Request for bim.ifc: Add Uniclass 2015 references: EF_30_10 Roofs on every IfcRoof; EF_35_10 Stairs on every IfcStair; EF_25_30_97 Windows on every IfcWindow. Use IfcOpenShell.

First a look at what the model holds.

```python
import ifcopenshell

model = ifcopenshell.open("bim.ifc")
print(model.schema)
print("classifications:", [c.Name for c in model.by_type("IfcClassification")])
for ifc_class in ("IfcDoor", "IfcRoof", "IfcStair", "IfcWall", "IfcWindow"):
    print(ifc_class, len(model.by_type(ifc_class)))
```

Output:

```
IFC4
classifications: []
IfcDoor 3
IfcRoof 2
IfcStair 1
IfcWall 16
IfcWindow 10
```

```python
import ifcopenshell
import ifcopenshell.api.classification

model = ifcopenshell.open("bim.ifc")

system = ifcopenshell.api.classification.add_classification(model, classification="Uniclass 2015")

codes = {
    "IfcRoof": ("EF_30_10", "Roofs"),
    "IfcStair": ("EF_35_10", "Stairs"),
    "IfcWindow": ("EF_25_30_97", "Windows"),
}
for ifc_class, (code, name) in codes.items():
    products = model.by_type(ifc_class)
    ifcopenshell.api.classification.add_reference(
        model, products=products, classification=system, identification=code, name=name
    )
    print(code, len(products))

model.write("bim_rev.ifc")
```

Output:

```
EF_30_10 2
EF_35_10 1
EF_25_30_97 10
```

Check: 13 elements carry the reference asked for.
